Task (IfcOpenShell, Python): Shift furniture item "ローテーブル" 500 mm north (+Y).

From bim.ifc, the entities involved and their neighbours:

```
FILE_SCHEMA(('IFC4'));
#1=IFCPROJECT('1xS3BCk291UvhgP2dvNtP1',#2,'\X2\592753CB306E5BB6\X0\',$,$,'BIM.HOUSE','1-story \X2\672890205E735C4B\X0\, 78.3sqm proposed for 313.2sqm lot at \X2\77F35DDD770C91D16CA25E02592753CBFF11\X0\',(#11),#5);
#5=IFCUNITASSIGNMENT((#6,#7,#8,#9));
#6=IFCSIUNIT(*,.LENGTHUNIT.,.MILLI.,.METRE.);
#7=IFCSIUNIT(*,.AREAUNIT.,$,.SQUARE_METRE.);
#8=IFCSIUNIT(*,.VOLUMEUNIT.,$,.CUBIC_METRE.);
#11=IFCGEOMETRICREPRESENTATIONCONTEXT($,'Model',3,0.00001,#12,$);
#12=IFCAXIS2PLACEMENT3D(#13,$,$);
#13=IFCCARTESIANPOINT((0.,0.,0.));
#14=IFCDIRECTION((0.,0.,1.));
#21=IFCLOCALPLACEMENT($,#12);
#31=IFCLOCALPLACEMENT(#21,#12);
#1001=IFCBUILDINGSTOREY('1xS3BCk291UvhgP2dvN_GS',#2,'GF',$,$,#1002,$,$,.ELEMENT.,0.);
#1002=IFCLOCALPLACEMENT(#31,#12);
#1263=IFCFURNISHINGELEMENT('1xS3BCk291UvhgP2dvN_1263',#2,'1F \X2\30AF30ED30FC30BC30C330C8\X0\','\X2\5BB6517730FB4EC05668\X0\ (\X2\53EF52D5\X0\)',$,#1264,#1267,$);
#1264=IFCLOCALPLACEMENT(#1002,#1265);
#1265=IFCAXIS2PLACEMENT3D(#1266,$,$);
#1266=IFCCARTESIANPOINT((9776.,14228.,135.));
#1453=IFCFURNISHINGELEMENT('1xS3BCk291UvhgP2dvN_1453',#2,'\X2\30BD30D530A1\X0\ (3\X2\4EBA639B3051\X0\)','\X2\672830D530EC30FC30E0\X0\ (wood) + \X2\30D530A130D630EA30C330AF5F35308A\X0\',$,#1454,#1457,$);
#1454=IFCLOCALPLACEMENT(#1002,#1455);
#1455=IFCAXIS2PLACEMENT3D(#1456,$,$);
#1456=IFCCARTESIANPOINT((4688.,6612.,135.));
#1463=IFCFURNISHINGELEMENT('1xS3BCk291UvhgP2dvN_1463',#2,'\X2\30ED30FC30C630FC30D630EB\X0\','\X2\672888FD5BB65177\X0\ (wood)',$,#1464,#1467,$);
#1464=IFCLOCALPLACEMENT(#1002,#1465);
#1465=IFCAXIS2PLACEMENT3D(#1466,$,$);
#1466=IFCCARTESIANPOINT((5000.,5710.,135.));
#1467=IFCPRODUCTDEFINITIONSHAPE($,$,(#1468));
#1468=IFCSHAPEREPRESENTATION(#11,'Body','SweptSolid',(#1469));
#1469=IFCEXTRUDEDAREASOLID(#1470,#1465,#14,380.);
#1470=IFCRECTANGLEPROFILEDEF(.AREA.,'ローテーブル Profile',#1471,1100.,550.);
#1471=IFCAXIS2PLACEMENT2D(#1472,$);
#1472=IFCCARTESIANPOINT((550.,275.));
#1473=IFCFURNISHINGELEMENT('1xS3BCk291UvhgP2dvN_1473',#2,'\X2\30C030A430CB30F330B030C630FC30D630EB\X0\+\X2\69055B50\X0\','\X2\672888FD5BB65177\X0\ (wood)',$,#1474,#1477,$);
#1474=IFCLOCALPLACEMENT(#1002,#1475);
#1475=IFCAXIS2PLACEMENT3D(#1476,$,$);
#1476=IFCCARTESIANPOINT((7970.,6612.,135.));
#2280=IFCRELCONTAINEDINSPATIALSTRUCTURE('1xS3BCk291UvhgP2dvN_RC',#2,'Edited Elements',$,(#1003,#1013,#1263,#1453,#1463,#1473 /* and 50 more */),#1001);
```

```python
import ifcopenshell
import ifcopenshell.api.geometry
import ifcopenshell.util.placement

model = ifcopenshell.open("bim.ifc")

item = model.by_id(1463)
matrix = ifcopenshell.util.placement.get_local_placement(item.ObjectPlacement)
matrix[1, 3] += 500.0
ifcopenshell.api.geometry.edit_object_placement(model, product=item, matrix=matrix, is_si=False)

print(ifcopenshell.util.placement.get_local_placement(item.ObjectPlacement).round(3) + 0.0)

model.write("bim_v2.ifc")
```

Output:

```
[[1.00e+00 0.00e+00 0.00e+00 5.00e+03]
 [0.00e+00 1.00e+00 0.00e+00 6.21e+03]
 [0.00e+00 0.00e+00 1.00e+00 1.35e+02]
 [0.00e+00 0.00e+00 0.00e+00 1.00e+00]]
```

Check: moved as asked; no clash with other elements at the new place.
